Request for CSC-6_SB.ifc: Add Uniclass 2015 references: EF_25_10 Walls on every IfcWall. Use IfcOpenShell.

First a look at what the model holds.

```python
import ifcopenshell

model = ifcopenshell.open("CSC-6_SB.ifc")
print(model.schema)
print("classifications:", [c.Name for c in model.by_type("IfcClassification")])
for ifc_class in ("IfcDoor", "IfcRoof", "IfcStair", "IfcWall", "IfcWindow"):
    print(ifc_class, len(model.by_type(ifc_class)))
```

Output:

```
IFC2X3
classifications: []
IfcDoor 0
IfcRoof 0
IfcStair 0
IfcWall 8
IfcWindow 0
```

```python
import ifcopenshell
import ifcopenshell.api.classification

model = ifcopenshell.open("CSC-6_SB.ifc")

# IFC2X3 requires Source and Edition and has no link from the project to the system.
system = model.create_entity("IfcClassification", Source="NBS", Edition="2015", Name="Uniclass 2015")

codes = {
    "IfcWall": ("EF_25_10", "Walls"),
}
for ifc_class, (code, name) in codes.items():
    products = model.by_type(ifc_class)
    ifcopenshell.api.classification.add_reference(
        model, products=products, classification=system, identification=code, name=name
    )
    print(code, len(products))

model.write("CSC-6_SB_v2.ifc")
```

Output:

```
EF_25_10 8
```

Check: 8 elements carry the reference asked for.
